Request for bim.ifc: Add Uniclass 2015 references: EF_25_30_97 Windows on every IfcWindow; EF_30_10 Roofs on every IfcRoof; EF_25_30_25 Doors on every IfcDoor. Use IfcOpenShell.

First a look at what the model holds.

```python
import ifcopenshell

model = ifcopenshell.open("bim.ifc")
print(model.schema)
print("classifications:", [c.Name for c in model.by_type("IfcClassification")])
for ifc_class in ("IfcDoor", "IfcRoof", "IfcStair", "IfcWall", "IfcWindow"):
    print(ifc_class, len(model.by_type(ifc_class)))
```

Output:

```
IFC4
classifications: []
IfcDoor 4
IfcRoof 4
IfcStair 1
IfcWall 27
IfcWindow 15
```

```python
import ifcopenshell
import ifcopenshell.api.classification

model = ifcopenshell.open("bim.ifc")

system = ifcopenshell.api.classification.add_classification(model, classification="Uniclass 2015")

codes = {
    "IfcWindow": ("EF_25_30_97", "Windows"),
    "IfcRoof": ("EF_30_10", "Roofs"),
    "IfcDoor": ("EF_25_30_25", "Doors"),
}
for ifc_class, (code, name) in codes.items():
    products = model.by_type(ifc_class)
    ifcopenshell.api.classification.add_reference(
        model, products=products, classification=system, identification=code, name=name
    )
    print(code, len(products))

model.write("bim-out.ifc")
```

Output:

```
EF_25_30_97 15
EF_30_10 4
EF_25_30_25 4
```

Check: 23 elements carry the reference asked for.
